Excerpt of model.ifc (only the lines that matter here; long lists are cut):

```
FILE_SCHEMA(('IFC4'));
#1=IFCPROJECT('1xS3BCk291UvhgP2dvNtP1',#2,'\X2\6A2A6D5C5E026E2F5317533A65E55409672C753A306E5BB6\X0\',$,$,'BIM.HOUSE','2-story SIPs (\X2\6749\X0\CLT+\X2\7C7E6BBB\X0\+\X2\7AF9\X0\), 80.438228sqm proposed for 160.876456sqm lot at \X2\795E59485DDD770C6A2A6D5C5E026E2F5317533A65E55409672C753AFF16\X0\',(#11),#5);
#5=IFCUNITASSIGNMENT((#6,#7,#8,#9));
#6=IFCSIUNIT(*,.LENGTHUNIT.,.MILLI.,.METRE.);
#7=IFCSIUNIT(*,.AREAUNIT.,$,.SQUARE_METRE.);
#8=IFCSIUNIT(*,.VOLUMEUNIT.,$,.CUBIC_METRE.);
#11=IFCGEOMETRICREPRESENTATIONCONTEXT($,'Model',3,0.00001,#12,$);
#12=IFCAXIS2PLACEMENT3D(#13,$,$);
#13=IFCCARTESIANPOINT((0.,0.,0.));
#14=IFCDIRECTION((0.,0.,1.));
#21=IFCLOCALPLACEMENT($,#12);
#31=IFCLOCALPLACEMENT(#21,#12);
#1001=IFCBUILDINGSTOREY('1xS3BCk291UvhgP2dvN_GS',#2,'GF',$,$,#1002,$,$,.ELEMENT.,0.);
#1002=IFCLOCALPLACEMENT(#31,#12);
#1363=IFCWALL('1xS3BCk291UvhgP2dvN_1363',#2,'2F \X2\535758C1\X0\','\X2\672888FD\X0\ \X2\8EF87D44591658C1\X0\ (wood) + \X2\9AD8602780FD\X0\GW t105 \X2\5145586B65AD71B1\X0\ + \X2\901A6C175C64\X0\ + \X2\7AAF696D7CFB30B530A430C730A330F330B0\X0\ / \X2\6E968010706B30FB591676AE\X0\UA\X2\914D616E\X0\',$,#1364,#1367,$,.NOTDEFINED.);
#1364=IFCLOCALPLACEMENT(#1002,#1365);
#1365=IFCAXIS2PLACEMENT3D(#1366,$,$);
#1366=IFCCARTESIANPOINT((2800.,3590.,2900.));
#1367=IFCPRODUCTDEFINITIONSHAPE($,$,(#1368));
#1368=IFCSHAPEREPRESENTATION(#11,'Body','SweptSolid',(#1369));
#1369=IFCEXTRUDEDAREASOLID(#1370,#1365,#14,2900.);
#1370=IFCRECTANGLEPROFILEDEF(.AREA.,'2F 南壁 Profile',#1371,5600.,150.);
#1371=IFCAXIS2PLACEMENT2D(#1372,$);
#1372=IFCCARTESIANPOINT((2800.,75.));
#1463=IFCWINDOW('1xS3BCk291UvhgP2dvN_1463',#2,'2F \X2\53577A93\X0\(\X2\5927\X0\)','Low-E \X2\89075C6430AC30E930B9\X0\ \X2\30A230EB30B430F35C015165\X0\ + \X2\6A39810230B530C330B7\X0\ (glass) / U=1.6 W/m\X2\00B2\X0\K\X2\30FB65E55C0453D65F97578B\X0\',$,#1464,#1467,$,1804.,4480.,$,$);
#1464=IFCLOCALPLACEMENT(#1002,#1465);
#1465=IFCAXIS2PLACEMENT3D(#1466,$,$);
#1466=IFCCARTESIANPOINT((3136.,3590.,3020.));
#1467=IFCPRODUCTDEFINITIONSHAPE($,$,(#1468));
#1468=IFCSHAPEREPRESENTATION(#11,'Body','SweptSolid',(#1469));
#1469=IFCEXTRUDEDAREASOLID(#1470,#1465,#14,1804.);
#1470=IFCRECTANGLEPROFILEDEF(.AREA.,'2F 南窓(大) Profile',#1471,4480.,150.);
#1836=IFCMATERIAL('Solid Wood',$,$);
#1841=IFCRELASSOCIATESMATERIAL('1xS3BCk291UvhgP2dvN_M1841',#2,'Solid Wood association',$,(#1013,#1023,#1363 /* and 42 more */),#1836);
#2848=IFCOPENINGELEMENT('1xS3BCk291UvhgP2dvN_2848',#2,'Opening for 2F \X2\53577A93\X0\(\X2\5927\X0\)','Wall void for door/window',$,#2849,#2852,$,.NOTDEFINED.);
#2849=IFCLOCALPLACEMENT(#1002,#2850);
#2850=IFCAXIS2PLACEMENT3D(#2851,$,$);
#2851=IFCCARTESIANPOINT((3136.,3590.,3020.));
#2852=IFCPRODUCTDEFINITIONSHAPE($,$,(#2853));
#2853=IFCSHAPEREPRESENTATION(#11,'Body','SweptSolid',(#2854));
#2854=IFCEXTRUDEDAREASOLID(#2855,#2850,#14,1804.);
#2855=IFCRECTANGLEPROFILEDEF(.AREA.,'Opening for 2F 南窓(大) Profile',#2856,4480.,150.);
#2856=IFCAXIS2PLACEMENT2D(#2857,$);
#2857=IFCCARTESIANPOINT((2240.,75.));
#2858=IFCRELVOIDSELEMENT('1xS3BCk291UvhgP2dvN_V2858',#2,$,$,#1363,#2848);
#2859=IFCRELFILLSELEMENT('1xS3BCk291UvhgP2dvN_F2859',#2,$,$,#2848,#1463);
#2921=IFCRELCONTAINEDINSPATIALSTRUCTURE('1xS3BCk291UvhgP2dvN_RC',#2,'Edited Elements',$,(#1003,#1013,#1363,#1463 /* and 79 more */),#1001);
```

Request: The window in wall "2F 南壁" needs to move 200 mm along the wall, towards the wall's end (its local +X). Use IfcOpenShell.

```python
import ifcopenshell
import ifcopenshell.api.geometry
import ifcopenshell.util.placement
import ifcopenshell.util.unit

model = ifcopenshell.open("model.ifc")
unit_scale = ifcopenshell.util.unit.calculate_unit_scale(model)

window = model.by_guid("1xS3BCk291UvhgP2dvN_1463")
opening = window.FillsVoids[0].RelatingOpeningElement
wall = opening.VoidsElements[0].RelatingBuildingElement

wall_matrix = ifcopenshell.util.placement.get_local_placement(wall.ObjectPlacement)
shift = wall_matrix[:3, 0] * 0.2 / unit_scale
before = ifcopenshell.util.placement.get_local_placement(window.ObjectPlacement)[:3, 3].copy()

# The window is not placed relative to its opening, so move both.
for product in (opening, window):
    matrix = ifcopenshell.util.placement.get_local_placement(product.ObjectPlacement)
    matrix[:3, 3] += shift
    ifcopenshell.api.geometry.edit_object_placement(model, product=product, matrix=matrix, is_si=False)

after = ifcopenshell.util.placement.get_local_placement(window.ObjectPlacement)[:3, 3]
print("window moved by", (after - before).round(3) + 0.0)

model.write("model_updated.ifc")
```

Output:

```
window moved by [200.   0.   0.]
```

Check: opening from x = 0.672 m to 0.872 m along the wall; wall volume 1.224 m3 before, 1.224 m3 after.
